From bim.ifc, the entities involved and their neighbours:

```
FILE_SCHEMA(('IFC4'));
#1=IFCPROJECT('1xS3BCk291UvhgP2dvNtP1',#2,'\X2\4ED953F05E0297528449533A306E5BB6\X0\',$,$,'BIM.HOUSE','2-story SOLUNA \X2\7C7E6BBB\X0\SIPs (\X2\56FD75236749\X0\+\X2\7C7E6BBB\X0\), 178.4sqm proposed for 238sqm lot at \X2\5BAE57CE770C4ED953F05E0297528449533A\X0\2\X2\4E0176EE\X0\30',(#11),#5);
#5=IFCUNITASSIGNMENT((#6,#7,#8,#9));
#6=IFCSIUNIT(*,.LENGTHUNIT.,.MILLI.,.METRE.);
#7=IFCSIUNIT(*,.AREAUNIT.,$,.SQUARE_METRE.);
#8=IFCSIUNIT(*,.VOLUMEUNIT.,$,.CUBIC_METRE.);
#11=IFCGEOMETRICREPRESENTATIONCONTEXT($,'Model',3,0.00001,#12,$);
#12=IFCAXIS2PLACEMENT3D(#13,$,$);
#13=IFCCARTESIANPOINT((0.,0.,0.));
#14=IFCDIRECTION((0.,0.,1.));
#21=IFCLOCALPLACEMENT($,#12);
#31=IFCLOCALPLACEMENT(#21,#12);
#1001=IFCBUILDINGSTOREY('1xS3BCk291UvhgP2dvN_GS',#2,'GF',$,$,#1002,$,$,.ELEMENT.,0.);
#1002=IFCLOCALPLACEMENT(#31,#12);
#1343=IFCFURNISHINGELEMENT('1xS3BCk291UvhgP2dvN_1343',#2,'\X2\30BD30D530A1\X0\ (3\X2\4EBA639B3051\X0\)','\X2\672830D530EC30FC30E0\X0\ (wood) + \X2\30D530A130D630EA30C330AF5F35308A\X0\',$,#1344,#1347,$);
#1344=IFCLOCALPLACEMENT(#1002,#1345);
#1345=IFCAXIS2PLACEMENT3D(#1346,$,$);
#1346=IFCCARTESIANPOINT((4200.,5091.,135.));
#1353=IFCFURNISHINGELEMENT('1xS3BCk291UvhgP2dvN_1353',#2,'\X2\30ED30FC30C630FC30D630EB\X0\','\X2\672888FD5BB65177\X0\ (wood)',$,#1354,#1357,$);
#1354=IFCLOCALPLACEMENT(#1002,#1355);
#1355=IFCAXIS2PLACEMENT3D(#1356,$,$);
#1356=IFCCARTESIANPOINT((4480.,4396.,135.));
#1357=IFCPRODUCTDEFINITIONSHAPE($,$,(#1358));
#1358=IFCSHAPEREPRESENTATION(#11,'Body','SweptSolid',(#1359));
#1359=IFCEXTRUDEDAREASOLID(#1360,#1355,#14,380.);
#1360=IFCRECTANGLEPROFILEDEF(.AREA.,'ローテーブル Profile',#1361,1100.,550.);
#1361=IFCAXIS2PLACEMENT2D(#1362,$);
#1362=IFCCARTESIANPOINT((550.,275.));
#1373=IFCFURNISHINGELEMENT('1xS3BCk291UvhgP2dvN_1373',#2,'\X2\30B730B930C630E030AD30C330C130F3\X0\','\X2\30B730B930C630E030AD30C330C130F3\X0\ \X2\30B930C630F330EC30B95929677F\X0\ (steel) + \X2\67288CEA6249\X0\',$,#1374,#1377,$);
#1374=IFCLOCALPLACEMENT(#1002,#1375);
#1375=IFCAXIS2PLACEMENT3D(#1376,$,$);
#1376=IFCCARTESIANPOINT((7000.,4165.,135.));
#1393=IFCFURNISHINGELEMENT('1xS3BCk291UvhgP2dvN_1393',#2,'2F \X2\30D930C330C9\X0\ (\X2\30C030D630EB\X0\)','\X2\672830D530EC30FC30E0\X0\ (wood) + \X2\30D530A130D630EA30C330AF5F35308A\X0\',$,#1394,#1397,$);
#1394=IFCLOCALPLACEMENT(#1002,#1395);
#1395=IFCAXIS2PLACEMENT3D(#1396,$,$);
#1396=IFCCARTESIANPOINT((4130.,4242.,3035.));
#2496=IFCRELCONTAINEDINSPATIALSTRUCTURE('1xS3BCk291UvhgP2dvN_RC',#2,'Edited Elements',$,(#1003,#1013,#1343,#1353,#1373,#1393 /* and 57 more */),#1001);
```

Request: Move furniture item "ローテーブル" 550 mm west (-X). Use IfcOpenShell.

```python
import ifcopenshell
import ifcopenshell.api.geometry
import ifcopenshell.util.placement

model = ifcopenshell.open("bim.ifc")

item = model.by_guid("1xS3BCk291UvhgP2dvN_1353")
matrix = ifcopenshell.util.placement.get_local_placement(item.ObjectPlacement)
matrix[0, 3] -= 550.0
ifcopenshell.api.geometry.edit_object_placement(model, product=item, matrix=matrix, is_si=False)

print(ifcopenshell.util.placement.get_local_placement(item.ObjectPlacement).round(3) + 0.0)

model.write("bim_rev.ifc")
```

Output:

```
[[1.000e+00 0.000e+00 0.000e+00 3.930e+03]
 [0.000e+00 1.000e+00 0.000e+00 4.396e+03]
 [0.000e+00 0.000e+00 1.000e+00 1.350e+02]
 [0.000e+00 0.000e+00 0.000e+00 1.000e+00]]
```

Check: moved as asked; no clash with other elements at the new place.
